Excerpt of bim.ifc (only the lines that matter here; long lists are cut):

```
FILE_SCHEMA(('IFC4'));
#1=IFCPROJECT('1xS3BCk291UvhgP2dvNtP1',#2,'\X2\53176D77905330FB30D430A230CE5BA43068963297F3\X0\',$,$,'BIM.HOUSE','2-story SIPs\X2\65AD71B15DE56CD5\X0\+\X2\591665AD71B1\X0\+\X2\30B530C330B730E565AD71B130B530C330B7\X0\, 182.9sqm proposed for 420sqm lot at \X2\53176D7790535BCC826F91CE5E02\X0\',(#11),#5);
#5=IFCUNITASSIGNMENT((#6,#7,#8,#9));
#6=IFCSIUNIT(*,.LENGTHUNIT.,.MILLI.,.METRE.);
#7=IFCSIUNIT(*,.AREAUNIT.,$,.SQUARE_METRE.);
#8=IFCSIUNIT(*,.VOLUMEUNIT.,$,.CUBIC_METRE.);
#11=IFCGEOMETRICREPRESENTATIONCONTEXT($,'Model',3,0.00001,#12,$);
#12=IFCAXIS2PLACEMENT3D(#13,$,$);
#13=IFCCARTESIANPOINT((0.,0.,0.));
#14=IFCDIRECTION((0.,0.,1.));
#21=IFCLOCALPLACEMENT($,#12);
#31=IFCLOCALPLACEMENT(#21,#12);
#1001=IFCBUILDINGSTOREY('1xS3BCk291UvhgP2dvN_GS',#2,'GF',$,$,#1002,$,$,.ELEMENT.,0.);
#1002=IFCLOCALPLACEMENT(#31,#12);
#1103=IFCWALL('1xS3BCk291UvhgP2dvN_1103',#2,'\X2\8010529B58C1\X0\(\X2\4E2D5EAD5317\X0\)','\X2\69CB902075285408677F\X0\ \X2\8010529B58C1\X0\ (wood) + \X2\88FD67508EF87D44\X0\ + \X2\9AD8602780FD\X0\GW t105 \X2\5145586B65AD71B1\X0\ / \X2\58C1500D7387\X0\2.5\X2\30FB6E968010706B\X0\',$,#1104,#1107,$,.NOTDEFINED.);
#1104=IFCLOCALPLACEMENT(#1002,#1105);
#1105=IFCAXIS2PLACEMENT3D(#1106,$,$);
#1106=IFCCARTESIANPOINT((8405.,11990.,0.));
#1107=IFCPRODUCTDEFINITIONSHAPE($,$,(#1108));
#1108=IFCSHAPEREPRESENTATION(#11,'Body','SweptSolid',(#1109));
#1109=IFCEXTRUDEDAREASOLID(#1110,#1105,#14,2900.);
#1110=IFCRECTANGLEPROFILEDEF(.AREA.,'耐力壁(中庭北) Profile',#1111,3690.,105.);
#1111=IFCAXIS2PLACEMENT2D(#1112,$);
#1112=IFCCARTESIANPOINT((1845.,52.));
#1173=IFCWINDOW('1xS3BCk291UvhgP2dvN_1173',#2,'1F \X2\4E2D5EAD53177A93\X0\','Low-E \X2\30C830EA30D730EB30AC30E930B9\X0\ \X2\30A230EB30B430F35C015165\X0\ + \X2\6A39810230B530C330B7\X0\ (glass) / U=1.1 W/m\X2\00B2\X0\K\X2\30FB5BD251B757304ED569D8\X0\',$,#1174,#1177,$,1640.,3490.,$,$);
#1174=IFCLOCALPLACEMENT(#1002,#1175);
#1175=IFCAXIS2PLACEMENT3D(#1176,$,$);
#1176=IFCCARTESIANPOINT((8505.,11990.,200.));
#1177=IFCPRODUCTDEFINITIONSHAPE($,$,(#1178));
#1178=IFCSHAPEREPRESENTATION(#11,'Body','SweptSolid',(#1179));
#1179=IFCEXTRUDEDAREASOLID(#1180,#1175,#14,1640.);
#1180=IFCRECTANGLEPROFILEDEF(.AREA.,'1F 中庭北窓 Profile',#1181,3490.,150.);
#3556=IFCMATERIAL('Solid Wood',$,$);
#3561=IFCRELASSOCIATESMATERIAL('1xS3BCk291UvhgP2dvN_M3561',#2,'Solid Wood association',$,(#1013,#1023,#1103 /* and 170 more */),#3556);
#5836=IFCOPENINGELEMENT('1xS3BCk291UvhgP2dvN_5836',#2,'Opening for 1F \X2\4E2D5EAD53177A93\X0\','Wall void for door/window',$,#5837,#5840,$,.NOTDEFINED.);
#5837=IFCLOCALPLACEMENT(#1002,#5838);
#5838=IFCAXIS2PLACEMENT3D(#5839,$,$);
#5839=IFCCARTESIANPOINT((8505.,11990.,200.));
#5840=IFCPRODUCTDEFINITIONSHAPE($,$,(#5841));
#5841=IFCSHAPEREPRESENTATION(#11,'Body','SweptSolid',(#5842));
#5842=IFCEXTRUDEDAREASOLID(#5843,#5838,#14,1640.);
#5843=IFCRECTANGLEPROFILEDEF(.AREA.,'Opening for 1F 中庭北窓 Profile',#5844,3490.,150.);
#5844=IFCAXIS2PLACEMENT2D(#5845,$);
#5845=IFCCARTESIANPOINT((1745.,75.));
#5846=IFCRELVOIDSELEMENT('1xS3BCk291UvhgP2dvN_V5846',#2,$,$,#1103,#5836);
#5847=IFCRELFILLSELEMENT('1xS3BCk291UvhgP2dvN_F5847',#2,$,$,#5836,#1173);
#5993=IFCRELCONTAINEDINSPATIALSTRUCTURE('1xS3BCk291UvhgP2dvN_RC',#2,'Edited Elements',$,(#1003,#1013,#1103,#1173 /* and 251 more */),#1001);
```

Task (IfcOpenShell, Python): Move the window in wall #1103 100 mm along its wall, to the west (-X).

```python
import ifcopenshell
import ifcopenshell.api.geometry
import ifcopenshell.util.placement
import ifcopenshell.util.unit

model = ifcopenshell.open("bim.ifc")
unit_scale = ifcopenshell.util.unit.calculate_unit_scale(model)

window = model.by_guid("1xS3BCk291UvhgP2dvN_1173")
opening = window.FillsVoids[0].RelatingOpeningElement
wall = opening.VoidsElements[0].RelatingBuildingElement

wall_matrix = ifcopenshell.util.placement.get_local_placement(wall.ObjectPlacement)
shift = wall_matrix[:3, 0] * -0.1 / unit_scale
before = ifcopenshell.util.placement.get_local_placement(window.ObjectPlacement)[:3, 3].copy()

# The window is not placed relative to its opening, so move both.
for product in (opening, window):
    matrix = ifcopenshell.util.placement.get_local_placement(product.ObjectPlacement)
    matrix[:3, 3] += shift
    ifcopenshell.api.geometry.edit_object_placement(model, product=product, matrix=matrix, is_si=False)

after = ifcopenshell.util.placement.get_local_placement(window.ObjectPlacement)[:3, 3]
print("window moved by", (after - before).round(3) + 0.0)

model.write("bim_v2.ifc")
```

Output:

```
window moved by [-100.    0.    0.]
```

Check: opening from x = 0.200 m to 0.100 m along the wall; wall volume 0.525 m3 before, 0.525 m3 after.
